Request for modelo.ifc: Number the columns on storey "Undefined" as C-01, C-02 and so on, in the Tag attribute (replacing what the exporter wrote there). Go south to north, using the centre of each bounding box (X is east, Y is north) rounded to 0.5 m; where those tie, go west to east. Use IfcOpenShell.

First a look at what the model holds.

```python
import ifcopenshell
import ifcopenshell.util.element
import ifcopenshell.util.placement

model = ifcopenshell.open("modelo.ifc")
print(model.schema)
storey = next(s for s in model.by_type("IfcBuildingStorey") if s.Name == "Undefined")
columns = [e for e in ifcopenshell.util.element.get_decomposition(storey) if e.is_a("IfcColumn")]
for e in sorted(columns, key=lambda e: e.id()):
    origin = ifcopenshell.util.placement.get_local_placement(e.ObjectPlacement)[:3, 3]
    print(e.id(), e.Tag, e.Name, origin.round(2) + 0.0, sep=" | ")
```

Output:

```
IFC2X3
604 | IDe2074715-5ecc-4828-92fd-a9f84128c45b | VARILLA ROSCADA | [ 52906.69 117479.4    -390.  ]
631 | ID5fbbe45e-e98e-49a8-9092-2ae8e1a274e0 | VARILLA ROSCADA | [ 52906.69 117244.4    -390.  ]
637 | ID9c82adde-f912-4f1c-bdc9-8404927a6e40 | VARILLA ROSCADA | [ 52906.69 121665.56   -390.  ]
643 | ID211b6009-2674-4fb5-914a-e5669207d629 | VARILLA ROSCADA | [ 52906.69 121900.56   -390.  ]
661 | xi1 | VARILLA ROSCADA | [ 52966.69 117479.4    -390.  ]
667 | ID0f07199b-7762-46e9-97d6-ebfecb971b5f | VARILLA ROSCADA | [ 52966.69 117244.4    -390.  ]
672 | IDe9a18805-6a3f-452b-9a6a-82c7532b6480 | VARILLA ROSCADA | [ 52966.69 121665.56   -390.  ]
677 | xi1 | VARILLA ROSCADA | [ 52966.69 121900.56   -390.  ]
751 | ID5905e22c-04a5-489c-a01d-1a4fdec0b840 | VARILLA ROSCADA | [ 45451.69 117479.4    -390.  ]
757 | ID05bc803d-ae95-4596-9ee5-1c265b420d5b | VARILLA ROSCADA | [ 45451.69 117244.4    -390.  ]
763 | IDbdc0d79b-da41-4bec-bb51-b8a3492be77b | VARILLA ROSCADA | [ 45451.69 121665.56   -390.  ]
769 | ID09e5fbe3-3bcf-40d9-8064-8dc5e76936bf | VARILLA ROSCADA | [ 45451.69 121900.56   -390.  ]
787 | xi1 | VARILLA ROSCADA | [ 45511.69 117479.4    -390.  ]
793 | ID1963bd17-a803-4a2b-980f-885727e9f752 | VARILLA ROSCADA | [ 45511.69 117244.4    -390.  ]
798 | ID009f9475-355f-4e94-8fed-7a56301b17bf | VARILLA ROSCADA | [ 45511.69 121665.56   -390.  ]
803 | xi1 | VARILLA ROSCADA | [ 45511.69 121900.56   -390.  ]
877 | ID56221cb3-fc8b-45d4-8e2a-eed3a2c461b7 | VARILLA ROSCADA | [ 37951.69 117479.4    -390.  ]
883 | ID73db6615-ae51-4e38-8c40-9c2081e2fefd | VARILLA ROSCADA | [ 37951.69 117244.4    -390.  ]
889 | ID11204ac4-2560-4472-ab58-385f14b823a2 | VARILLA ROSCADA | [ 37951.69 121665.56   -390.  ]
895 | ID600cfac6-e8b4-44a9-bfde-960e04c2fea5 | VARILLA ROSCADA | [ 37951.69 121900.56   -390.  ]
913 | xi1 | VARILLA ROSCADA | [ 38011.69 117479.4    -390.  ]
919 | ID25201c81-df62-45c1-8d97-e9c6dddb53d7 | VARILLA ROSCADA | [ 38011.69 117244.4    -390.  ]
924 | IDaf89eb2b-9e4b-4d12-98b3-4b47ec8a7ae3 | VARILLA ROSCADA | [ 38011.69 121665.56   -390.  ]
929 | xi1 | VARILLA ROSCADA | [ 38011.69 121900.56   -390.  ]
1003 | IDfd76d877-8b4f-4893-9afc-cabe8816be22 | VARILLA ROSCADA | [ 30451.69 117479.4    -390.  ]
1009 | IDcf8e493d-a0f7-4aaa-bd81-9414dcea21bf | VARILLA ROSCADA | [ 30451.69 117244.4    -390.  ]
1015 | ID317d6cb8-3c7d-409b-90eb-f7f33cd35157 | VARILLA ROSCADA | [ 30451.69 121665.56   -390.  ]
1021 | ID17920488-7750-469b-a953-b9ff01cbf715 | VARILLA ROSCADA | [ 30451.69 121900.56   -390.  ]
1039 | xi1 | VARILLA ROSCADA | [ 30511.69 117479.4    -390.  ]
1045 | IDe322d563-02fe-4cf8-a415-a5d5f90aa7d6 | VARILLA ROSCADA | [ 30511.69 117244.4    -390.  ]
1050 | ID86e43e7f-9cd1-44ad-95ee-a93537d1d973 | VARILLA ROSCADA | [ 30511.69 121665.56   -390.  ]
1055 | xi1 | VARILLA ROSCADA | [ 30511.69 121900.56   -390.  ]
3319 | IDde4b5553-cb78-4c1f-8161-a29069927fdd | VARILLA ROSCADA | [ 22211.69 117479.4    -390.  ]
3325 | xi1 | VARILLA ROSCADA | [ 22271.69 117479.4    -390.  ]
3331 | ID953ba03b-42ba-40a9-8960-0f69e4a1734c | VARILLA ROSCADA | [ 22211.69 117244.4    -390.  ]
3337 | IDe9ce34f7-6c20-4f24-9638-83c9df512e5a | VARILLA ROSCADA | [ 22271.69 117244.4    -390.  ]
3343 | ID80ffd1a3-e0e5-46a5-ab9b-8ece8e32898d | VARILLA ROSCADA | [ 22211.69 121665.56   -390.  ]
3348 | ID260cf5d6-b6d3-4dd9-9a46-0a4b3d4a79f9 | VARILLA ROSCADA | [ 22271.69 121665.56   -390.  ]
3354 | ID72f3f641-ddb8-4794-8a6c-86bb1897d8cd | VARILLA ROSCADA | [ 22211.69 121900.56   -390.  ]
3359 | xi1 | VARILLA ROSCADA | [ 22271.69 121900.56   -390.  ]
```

```python
import ifcopenshell
import ifcopenshell.geom
import ifcopenshell.util.element
import ifcopenshell.util.shape

model = ifcopenshell.open("modelo.ifc")
settings = ifcopenshell.geom.settings()
settings.set("use-world-coords", True)


def centre(element):
    shape = ifcopenshell.geom.create_shape(settings, element)
    return ifcopenshell.util.shape.get_bbox_centroid(shape.geometry)


storey = next(s for s in model.by_type("IfcBuildingStorey") if s.Name == "Undefined")
columns = [e for e in ifcopenshell.util.element.get_decomposition(storey) if e.is_a("IfcColumn")]

# Insertion points can sit at a corner or the storey origin, so sort by the geometry (in metres).
centres = {e: centre(e) for e in columns}
columns.sort(key=lambda e: (round(centres[e][1] / 0.5), centres[e][0]))

for i, e in enumerate(columns, start=1):
    number = f"C-{i:02d}"
    e.Tag = number
    print(e.id(), number)

model.write("modelo_updated.ifc")
```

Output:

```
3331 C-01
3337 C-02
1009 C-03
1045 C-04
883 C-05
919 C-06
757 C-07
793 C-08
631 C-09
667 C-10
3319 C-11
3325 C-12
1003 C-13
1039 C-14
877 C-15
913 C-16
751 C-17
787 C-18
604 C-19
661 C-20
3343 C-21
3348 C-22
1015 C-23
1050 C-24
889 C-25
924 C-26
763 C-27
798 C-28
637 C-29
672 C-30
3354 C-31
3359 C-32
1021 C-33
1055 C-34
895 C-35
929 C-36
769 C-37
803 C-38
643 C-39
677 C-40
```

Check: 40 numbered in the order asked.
